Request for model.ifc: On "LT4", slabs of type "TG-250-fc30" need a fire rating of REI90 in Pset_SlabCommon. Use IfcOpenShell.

First a look at what the model holds.

```python
import ifcopenshell
import ifcopenshell.util.element

model = ifcopenshell.open("model.ifc")
print(model.schema)
storey = next(s for s in model.by_type("IfcBuildingStorey") if s.Name == "LT4")
slabs = [e for e in ifcopenshell.util.element.get_decomposition(storey) if e.is_a("IfcSlab")]
seen = {}
for e in slabs:
    element_type = ifcopenshell.util.element.get_type(e)
    key = (element_type.Name if element_type != e and element_type else None, ifcopenshell.util.element.get_pset(e, "Pset_SlabCommon", "FireRating"))
    seen[key] = seen.get(key, 0) + 1
for (name, value), count in sorted(seen.items(), key=str):
    print(count, "x", name, "|", value)
```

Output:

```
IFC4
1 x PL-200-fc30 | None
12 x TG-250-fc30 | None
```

```python
import ifcopenshell
import ifcopenshell.api.pset
import ifcopenshell.util.element

model = ifcopenshell.open("model.ifc")

storey = next(s for s in model.by_type("IfcBuildingStorey") if s.Name == "LT4")
slabs = [e for e in ifcopenshell.util.element.get_decomposition(storey) if e.is_a("IfcSlab")]

count = 0
for e in slabs:
    element_type = ifcopenshell.util.element.get_type(e)
    if element_type in (None, e) or element_type.Name != "TG-250-fc30":
        continue
    # add_pset returns the element's existing set when there is one.
    pset = ifcopenshell.api.pset.add_pset(model, product=e, name="Pset_SlabCommon")
    ifcopenshell.api.pset.edit_pset(model, pset=pset, properties={"FireRating": "REI90"})
    count += 1

print(count, "slabs updated")

model.write("model_edited.ifc")
```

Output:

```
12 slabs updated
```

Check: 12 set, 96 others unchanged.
